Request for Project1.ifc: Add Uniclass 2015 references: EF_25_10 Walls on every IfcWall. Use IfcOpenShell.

First a look at what the model holds.

```python
import ifcopenshell

model = ifcopenshell.open("Project1.ifc")
print(model.schema)
print("classifications:", [c.Name for c in model.by_type("IfcClassification")])
for ifc_class in ("IfcDoor", "IfcRoof", "IfcStair", "IfcWall", "IfcWindow"):
    print(ifc_class, len(model.by_type(ifc_class)))
```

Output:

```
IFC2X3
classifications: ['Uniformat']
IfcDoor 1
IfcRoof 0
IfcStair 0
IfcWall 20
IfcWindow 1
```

```python
import ifcopenshell
import ifcopenshell.api.classification

model = ifcopenshell.open("Project1.ifc")

# IFC2X3 requires Source and Edition and has no link from the project to the system.
system = model.create_entity("IfcClassification", Source="NBS", Edition="2015", Name="Uniclass 2015")

codes = {
    "IfcWall": ("EF_25_10", "Walls"),
}
for ifc_class, (code, name) in codes.items():
    products = model.by_type(ifc_class)
    ifcopenshell.api.classification.add_reference(
        model, products=products, classification=system, identification=code, name=name
    )
    print(code, len(products))

model.write("Project1_rev.ifc")
```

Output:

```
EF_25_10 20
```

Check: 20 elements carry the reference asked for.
